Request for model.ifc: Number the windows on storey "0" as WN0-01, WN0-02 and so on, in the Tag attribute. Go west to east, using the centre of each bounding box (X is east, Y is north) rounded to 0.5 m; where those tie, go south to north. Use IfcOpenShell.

First a look at what the model holds.

```python
import ifcopenshell
import ifcopenshell.util.element
import ifcopenshell.util.placement

model = ifcopenshell.open("model.ifc")
print(model.schema)
storey = next(s for s in model.by_type("IfcBuildingStorey") if s.Name == "0")
windows = [e for e in ifcopenshell.util.element.get_decomposition(storey) if e.is_a("IfcWindow")]
for e in sorted(windows, key=lambda e: e.id()):
    origin = ifcopenshell.util.placement.get_local_placement(e.ObjectPlacement)[:3, 3]
    print(e.id(), e.Tag, e.Name, origin.round(2) + 0.0, sep=" | ")
```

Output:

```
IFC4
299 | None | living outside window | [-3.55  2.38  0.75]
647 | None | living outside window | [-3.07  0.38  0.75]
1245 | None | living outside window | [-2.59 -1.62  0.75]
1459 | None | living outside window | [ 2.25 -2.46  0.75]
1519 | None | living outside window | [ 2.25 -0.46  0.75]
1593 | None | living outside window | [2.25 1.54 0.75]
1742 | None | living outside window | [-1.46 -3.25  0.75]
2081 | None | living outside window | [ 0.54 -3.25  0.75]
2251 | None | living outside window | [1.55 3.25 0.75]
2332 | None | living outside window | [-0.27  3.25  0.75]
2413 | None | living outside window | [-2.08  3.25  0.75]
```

```python
import ifcopenshell
import ifcopenshell.geom
import ifcopenshell.util.element
import ifcopenshell.util.shape

model = ifcopenshell.open("model.ifc")
settings = ifcopenshell.geom.settings()
settings.set("use-world-coords", True)


def centre(element):
    shape = ifcopenshell.geom.create_shape(settings, element)
    return ifcopenshell.util.shape.get_bbox_centroid(shape.geometry)


storey = next(s for s in model.by_type("IfcBuildingStorey") if s.Name == "0")
windows = [e for e in ifcopenshell.util.element.get_decomposition(storey) if e.is_a("IfcWindow")]

# Insertion points can sit at a corner or the storey origin, so sort by the geometry (in metres).
centres = {e: centre(e) for e in windows}
windows.sort(key=lambda e: (round(centres[e][0] / 0.5), centres[e][1]))

for i, e in enumerate(windows, start=1):
    number = f"WN0-{i:02d}"
    e.Tag = number
    print(e.id(), number)

model.write("model_rev.ifc")
```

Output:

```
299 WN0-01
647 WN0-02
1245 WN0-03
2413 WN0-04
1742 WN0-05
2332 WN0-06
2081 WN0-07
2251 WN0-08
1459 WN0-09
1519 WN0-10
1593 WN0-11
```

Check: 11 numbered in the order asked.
